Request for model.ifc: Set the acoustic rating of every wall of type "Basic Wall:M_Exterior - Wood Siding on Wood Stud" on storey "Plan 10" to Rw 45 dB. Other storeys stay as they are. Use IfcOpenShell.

First a look at what the model holds.

```python
import ifcopenshell
import ifcopenshell.util.element

model = ifcopenshell.open("model.ifc")
print(model.schema)
storey = next(s for s in model.by_type("IfcBuildingStorey") if s.Name == "Plan 10")
walls = [e for e in ifcopenshell.util.element.get_decomposition(storey) if e.is_a("IfcWall")]
seen = {}
for e in walls:
    element_type = ifcopenshell.util.element.get_type(e)
    key = (element_type.Name if element_type != e and element_type else None, ifcopenshell.util.element.get_pset(e, "Pset_WallCommon", "AcousticRating"))
    seen[key] = seen.get(key, 0) + 1
for (name, value), count in sorted(seen.items(), key=str):
    print(count, "x", name, "|", value)
```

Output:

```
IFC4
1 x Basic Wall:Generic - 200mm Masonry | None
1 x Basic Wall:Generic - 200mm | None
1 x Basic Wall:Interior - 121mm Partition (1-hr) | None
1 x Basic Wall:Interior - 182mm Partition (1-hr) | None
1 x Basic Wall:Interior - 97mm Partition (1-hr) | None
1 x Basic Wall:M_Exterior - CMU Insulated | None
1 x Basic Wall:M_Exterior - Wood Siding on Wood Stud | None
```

```python
import ifcopenshell
import ifcopenshell.api.pset
import ifcopenshell.util.element

model = ifcopenshell.open("model.ifc")

storey = next(s for s in model.by_type("IfcBuildingStorey") if s.Name == "Plan 10")
walls = [e for e in ifcopenshell.util.element.get_decomposition(storey) if e.is_a("IfcWall")]

count = 0
for e in walls:
    element_type = ifcopenshell.util.element.get_type(e)
    if element_type in (None, e) or element_type.Name != "Basic Wall:M_Exterior - Wood Siding on Wood Stud":
        continue
    # add_pset returns the element's existing set when there is one.
    pset = ifcopenshell.api.pset.add_pset(model, product=e, name="Pset_WallCommon")
    ifcopenshell.api.pset.edit_pset(model, pset=pset, properties={"AcousticRating": "Rw 45 dB"})
    count += 1

print(count, "walls updated")

model.write("model_v2.ifc")
```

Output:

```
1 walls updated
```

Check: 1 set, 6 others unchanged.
